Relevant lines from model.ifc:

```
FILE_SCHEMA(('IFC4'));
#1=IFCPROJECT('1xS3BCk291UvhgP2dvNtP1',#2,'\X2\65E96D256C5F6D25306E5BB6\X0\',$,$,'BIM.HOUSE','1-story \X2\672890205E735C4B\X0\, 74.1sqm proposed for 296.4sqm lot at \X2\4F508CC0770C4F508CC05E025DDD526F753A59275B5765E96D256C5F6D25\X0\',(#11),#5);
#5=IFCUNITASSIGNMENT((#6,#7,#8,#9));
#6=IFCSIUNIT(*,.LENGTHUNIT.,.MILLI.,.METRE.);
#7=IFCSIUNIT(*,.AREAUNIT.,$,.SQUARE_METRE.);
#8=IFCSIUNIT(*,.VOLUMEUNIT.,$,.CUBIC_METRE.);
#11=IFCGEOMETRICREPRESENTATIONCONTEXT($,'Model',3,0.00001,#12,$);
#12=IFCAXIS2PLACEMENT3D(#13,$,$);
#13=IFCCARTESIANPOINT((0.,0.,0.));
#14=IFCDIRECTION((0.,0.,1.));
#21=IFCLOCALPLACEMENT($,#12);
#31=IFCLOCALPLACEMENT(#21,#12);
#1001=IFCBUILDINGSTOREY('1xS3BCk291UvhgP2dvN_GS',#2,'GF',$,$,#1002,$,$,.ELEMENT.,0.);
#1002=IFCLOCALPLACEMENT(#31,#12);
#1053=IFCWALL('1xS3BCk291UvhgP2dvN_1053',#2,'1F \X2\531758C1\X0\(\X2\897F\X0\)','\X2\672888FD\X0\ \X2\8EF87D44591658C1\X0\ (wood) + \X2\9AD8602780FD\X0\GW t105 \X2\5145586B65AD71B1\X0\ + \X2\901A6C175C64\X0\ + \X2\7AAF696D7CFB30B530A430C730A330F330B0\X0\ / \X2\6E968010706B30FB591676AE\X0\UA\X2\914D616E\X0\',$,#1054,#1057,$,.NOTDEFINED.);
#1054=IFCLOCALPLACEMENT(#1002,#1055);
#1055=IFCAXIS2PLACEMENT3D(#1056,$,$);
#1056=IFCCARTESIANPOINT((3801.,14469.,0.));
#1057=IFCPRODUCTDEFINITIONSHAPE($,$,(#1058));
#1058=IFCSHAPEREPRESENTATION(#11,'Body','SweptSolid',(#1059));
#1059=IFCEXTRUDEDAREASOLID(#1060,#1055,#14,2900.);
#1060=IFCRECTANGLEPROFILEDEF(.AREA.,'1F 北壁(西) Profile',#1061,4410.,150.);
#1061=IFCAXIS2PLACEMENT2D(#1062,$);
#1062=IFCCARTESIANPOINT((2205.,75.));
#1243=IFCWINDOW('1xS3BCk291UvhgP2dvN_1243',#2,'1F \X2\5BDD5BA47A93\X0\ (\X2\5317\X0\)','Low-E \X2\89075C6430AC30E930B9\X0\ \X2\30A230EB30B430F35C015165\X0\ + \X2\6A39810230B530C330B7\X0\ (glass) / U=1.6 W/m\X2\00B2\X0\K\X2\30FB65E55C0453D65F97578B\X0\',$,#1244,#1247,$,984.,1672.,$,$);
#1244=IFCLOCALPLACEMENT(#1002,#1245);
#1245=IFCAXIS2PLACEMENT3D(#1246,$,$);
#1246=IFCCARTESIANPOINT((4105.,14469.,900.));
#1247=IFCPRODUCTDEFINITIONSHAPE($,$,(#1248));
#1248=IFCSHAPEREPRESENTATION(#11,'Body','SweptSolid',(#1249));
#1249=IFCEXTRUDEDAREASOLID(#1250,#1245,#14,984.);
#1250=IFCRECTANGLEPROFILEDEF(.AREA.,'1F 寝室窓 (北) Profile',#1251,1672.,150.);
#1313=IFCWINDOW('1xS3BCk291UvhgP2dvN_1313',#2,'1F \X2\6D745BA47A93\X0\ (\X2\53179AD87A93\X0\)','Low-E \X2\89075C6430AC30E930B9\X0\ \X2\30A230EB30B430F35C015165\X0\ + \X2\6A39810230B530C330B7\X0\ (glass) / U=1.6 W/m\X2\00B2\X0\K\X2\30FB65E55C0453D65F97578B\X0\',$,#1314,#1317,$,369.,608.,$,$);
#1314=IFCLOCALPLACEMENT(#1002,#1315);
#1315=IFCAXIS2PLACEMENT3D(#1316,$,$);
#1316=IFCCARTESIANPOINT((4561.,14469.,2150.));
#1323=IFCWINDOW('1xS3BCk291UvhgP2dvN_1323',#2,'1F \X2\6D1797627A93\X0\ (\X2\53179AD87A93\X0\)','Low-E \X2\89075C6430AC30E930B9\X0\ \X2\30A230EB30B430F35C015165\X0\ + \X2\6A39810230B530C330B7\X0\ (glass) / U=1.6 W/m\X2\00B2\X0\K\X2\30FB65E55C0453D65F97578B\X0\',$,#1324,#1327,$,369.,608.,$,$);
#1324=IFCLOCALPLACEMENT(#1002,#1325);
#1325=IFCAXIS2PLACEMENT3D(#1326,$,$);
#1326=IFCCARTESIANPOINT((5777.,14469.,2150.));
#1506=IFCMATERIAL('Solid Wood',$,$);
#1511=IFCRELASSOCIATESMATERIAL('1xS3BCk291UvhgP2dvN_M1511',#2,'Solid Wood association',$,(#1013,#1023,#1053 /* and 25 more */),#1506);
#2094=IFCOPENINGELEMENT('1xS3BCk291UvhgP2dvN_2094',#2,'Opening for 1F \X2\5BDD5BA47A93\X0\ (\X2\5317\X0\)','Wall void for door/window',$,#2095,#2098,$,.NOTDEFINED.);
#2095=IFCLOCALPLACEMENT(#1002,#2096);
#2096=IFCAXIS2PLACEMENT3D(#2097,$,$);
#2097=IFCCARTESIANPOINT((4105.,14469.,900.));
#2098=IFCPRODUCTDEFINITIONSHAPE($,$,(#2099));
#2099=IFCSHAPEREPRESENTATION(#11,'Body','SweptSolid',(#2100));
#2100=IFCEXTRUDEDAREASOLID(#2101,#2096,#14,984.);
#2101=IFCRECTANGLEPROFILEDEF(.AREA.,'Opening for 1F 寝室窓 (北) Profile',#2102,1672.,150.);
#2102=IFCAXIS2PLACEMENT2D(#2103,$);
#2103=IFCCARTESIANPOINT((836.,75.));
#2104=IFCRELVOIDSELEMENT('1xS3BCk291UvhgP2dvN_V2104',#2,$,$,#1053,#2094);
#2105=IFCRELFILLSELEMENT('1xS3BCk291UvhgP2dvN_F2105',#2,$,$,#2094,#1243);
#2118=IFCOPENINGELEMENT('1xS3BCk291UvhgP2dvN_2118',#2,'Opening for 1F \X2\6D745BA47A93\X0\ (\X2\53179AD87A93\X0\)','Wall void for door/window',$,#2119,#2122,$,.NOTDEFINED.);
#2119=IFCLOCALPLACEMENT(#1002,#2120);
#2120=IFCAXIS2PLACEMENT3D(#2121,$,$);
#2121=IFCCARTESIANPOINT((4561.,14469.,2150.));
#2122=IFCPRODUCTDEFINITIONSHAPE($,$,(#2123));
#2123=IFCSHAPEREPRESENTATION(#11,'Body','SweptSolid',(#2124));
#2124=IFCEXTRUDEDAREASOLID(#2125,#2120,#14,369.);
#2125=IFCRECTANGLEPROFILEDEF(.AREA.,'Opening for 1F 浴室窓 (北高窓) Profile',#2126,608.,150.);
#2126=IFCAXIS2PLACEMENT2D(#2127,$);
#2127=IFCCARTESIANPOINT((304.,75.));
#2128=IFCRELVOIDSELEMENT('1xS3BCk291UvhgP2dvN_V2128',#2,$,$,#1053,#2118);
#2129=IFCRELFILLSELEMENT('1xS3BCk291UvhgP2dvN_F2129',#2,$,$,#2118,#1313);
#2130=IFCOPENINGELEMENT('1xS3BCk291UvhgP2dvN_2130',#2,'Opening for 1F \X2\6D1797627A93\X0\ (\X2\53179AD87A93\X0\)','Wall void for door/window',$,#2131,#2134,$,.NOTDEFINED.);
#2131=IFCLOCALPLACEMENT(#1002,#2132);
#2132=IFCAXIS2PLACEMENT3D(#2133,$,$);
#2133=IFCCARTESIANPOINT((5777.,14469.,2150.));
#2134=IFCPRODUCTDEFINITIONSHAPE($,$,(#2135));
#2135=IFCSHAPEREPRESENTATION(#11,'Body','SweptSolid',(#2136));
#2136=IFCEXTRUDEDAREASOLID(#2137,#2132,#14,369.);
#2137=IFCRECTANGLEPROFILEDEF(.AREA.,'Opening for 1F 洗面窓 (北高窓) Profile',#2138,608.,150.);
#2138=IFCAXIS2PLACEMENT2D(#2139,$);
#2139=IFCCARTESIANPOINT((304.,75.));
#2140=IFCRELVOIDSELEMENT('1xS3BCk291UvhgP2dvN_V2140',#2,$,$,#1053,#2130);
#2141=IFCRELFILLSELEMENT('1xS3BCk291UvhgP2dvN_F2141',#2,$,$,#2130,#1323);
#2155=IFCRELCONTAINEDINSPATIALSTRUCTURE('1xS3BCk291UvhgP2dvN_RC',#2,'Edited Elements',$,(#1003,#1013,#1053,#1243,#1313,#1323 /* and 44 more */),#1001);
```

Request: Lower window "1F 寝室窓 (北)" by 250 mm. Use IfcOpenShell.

```python
import numpy as np
import ifcopenshell
import ifcopenshell.api.geometry
import ifcopenshell.util.placement
import ifcopenshell.util.unit

model = ifcopenshell.open("model.ifc")
unit_scale = ifcopenshell.util.unit.calculate_unit_scale(model)

window = model.by_guid("1xS3BCk291UvhgP2dvN_1243")
opening = window.FillsVoids[0].RelatingOpeningElement
dz = -250.0

shift = np.array([0.0, 0.0, dz])
# The window is not placed relative to its opening, so move both.
for product in (opening, window):
    matrix = ifcopenshell.util.placement.get_local_placement(product.ObjectPlacement)
    matrix[:3, 3] += shift
    ifcopenshell.api.geometry.edit_object_placement(model, product=product, matrix=matrix, is_si=False)

print(f"moved by {dz * unit_scale:+.3f} m")

model.write("model_rev.ifc")
```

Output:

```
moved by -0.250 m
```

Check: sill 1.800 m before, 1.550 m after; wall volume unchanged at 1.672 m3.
